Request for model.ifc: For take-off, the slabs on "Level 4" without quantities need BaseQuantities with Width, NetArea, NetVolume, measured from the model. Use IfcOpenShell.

First a look at what the model holds.

```python
import ifcopenshell
import ifcopenshell.util.element
import ifcopenshell.util.unit

model = ifcopenshell.open("model.ifc")
print(model.schema)
for unit_type in ("LENGTHUNIT", "AREAUNIT", "VOLUMEUNIT"):
    print(unit_type, ifcopenshell.util.unit.calculate_unit_scale(model, unit_type))
storey = next(s for s in model.by_type("IfcBuildingStorey") if s.Name == "Level 4")
slabs = [e for e in ifcopenshell.util.element.get_decomposition(storey) if e.is_a("IfcSlab")]
for e in sorted(slabs, key=lambda e: e.id()):
    print(e.id(), e.is_a(), e.Name, list(ifcopenshell.util.element.get_psets(e, qtos_only=True)), sep=" | ")
```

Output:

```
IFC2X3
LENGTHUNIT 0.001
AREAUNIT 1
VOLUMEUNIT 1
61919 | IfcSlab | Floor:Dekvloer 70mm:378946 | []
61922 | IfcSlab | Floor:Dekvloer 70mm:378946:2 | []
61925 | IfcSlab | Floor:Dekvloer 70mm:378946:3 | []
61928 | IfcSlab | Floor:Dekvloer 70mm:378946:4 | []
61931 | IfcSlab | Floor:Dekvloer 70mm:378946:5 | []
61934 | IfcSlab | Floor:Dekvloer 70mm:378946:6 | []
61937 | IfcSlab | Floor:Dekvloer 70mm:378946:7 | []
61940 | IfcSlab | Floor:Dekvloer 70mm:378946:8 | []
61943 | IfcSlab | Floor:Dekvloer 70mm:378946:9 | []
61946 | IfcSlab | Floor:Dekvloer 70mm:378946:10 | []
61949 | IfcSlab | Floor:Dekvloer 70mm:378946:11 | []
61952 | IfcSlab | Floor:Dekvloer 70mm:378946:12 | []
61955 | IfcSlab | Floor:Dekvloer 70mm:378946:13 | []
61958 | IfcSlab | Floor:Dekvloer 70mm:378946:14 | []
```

```python
import ifcopenshell
import ifcopenshell.api.pset
import ifcopenshell.geom
import ifcopenshell.util.element
import ifcopenshell.util.shape
import ifcopenshell.util.unit

model = ifcopenshell.open("model.ifc")
unit_scale = ifcopenshell.util.unit.calculate_unit_scale(model)
area_scale = ifcopenshell.util.unit.calculate_unit_scale(model, "AREAUNIT")
volume_scale = ifcopenshell.util.unit.calculate_unit_scale(model, "VOLUMEUNIT")
settings = ifcopenshell.geom.settings()

storey = next(s for s in model.by_type("IfcBuildingStorey") if s.Name == "Level 4")
slabs = [e for e in ifcopenshell.util.element.get_decomposition(storey) if e.is_a("IfcSlab")]

for e in sorted(slabs, key=lambda e: e.id()):
    if ifcopenshell.util.element.get_psets(e, qtos_only=True, should_inherit=False):
        continue
    # Geometry comes back in metres, in the element's own axes.
    shape = ifcopenshell.geom.create_shape(settings, e)
    values = {
        "Width": ifcopenshell.util.shape.get_z(shape.geometry) / unit_scale,
        "NetArea": ifcopenshell.util.shape.get_footprint_area(shape.geometry) / area_scale,
        "NetVolume": ifcopenshell.util.shape.get_volume(shape.geometry) / volume_scale,
    }
    qto = ifcopenshell.api.pset.add_qto(model, product=e, name="BaseQuantities")
    ifcopenshell.api.pset.edit_qto(model, qto=qto, properties=values)
    print(e.id(), {k: round(v, 3) for k, v in values.items()})

model.write("model_updated.ifc")
```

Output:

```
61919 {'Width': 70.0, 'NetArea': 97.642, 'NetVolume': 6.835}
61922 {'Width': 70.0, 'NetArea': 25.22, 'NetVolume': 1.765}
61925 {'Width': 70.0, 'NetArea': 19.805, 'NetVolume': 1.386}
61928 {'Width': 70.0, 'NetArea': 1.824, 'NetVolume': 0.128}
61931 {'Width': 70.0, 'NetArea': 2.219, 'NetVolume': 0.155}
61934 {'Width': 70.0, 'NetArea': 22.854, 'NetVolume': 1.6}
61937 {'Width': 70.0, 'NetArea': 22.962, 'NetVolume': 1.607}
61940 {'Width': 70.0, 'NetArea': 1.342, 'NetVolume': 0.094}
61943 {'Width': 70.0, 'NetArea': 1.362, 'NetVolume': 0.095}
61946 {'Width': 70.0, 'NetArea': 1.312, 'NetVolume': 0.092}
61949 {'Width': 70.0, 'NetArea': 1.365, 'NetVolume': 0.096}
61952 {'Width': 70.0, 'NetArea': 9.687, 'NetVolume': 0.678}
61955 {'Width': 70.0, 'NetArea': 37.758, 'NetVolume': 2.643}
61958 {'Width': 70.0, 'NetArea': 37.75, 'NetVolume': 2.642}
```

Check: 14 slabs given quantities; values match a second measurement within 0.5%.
